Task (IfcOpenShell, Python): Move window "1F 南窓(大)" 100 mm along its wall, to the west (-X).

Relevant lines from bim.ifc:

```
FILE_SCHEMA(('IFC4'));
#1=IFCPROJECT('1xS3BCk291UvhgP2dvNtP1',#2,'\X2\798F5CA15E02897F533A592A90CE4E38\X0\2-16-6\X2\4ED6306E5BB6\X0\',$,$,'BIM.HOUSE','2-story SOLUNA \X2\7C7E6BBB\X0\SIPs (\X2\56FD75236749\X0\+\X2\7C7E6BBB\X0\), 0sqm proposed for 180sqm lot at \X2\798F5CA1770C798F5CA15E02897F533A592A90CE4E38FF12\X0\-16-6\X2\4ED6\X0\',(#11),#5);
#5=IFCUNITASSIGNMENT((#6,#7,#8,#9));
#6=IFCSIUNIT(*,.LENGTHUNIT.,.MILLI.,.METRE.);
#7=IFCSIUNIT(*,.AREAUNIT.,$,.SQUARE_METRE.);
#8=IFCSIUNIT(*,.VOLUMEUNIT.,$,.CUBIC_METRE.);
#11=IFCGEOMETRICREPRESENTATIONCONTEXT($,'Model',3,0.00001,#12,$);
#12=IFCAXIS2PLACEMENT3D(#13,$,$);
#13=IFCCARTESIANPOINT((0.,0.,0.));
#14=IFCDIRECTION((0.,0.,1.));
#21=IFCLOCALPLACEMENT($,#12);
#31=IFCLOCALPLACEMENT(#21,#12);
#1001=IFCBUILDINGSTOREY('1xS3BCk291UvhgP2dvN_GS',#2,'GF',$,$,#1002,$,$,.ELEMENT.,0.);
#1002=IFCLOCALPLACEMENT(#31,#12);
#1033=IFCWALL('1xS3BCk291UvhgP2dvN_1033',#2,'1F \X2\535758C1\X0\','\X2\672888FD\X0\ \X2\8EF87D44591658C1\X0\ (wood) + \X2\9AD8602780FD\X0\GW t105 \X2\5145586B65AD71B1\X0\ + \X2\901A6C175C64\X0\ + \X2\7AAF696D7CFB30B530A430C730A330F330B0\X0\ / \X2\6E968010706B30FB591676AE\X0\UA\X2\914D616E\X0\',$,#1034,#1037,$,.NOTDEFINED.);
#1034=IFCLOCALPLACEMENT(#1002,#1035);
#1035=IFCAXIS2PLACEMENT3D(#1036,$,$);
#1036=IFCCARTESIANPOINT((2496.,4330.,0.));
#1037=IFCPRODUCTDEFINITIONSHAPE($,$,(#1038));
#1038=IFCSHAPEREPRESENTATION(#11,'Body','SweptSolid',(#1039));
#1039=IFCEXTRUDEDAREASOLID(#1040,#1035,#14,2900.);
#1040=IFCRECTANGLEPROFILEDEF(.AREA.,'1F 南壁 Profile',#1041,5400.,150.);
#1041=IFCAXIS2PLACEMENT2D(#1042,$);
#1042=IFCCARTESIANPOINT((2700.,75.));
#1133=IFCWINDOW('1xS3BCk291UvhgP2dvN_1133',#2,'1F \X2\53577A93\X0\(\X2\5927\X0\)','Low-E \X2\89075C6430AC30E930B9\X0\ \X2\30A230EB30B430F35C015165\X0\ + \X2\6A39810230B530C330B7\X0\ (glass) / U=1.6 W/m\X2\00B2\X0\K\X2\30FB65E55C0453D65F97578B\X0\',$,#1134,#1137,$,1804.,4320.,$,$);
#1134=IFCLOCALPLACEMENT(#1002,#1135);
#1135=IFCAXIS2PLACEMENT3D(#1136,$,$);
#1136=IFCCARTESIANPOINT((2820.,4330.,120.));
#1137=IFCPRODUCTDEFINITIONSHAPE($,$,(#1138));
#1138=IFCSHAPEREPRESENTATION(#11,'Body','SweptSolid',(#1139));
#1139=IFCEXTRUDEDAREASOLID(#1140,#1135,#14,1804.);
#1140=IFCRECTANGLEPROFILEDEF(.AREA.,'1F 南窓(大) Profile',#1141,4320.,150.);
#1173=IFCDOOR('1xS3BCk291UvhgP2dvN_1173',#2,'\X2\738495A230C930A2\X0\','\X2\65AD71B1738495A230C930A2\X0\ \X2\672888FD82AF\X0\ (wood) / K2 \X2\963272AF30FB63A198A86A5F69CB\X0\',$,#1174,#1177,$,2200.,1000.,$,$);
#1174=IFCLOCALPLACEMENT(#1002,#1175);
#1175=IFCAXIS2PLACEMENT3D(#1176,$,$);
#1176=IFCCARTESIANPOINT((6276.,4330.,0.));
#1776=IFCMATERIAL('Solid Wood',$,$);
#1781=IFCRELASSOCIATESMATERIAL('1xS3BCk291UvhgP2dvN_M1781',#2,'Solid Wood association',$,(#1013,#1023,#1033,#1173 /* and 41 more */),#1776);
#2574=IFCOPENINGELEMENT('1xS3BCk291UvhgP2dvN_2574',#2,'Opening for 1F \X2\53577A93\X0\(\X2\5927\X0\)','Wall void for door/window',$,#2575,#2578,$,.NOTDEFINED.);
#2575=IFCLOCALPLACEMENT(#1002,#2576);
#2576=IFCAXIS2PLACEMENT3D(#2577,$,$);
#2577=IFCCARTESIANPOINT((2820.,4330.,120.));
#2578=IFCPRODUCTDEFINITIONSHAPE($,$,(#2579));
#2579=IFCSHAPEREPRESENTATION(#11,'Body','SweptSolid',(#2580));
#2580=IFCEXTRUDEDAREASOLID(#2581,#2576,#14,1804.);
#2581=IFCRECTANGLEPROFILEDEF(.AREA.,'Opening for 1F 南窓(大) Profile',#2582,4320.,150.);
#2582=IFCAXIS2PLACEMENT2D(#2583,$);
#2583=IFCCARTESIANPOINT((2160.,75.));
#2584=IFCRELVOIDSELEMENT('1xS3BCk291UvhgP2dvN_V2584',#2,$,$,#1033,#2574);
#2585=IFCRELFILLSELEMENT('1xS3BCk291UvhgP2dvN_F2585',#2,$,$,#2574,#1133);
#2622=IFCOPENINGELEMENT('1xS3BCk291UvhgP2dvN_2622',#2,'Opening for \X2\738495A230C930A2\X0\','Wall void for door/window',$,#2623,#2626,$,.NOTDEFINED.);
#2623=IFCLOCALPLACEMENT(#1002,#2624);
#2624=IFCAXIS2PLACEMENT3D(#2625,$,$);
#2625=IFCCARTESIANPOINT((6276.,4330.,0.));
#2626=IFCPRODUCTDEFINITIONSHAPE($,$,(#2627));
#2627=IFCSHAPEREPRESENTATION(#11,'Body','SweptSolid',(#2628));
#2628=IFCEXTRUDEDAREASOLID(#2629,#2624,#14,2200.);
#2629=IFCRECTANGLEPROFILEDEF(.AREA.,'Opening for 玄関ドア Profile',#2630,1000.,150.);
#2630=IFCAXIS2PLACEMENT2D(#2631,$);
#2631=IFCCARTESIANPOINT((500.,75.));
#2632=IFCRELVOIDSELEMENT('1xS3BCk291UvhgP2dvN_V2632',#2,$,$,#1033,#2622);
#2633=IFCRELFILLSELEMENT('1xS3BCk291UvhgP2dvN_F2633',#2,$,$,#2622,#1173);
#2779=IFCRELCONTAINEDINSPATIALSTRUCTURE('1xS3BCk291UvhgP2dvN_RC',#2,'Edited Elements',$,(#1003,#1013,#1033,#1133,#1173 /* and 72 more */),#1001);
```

```python
import ifcopenshell
import ifcopenshell.api.geometry
import ifcopenshell.util.placement
import ifcopenshell.util.unit

model = ifcopenshell.open("bim.ifc")
unit_scale = ifcopenshell.util.unit.calculate_unit_scale(model)

window = model.by_id(1133)
opening = window.FillsVoids[0].RelatingOpeningElement
wall = opening.VoidsElements[0].RelatingBuildingElement

wall_matrix = ifcopenshell.util.placement.get_local_placement(wall.ObjectPlacement)
shift = wall_matrix[:3, 0] * -0.1 / unit_scale
before = ifcopenshell.util.placement.get_local_placement(window.ObjectPlacement)[:3, 3].copy()

# The window is not placed relative to its opening, so move both.
for product in (opening, window):
    matrix = ifcopenshell.util.placement.get_local_placement(product.ObjectPlacement)
    matrix[:3, 3] += shift
    ifcopenshell.api.geometry.edit_object_placement(model, product=product, matrix=matrix, is_si=False)

after = ifcopenshell.util.placement.get_local_placement(window.ObjectPlacement)[:3, 3]
print("window moved by", (after - before).round(3) + 0.0)

model.write("bim_rev.ifc")
```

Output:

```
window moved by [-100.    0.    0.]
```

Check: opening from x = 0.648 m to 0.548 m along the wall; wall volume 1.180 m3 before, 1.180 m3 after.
